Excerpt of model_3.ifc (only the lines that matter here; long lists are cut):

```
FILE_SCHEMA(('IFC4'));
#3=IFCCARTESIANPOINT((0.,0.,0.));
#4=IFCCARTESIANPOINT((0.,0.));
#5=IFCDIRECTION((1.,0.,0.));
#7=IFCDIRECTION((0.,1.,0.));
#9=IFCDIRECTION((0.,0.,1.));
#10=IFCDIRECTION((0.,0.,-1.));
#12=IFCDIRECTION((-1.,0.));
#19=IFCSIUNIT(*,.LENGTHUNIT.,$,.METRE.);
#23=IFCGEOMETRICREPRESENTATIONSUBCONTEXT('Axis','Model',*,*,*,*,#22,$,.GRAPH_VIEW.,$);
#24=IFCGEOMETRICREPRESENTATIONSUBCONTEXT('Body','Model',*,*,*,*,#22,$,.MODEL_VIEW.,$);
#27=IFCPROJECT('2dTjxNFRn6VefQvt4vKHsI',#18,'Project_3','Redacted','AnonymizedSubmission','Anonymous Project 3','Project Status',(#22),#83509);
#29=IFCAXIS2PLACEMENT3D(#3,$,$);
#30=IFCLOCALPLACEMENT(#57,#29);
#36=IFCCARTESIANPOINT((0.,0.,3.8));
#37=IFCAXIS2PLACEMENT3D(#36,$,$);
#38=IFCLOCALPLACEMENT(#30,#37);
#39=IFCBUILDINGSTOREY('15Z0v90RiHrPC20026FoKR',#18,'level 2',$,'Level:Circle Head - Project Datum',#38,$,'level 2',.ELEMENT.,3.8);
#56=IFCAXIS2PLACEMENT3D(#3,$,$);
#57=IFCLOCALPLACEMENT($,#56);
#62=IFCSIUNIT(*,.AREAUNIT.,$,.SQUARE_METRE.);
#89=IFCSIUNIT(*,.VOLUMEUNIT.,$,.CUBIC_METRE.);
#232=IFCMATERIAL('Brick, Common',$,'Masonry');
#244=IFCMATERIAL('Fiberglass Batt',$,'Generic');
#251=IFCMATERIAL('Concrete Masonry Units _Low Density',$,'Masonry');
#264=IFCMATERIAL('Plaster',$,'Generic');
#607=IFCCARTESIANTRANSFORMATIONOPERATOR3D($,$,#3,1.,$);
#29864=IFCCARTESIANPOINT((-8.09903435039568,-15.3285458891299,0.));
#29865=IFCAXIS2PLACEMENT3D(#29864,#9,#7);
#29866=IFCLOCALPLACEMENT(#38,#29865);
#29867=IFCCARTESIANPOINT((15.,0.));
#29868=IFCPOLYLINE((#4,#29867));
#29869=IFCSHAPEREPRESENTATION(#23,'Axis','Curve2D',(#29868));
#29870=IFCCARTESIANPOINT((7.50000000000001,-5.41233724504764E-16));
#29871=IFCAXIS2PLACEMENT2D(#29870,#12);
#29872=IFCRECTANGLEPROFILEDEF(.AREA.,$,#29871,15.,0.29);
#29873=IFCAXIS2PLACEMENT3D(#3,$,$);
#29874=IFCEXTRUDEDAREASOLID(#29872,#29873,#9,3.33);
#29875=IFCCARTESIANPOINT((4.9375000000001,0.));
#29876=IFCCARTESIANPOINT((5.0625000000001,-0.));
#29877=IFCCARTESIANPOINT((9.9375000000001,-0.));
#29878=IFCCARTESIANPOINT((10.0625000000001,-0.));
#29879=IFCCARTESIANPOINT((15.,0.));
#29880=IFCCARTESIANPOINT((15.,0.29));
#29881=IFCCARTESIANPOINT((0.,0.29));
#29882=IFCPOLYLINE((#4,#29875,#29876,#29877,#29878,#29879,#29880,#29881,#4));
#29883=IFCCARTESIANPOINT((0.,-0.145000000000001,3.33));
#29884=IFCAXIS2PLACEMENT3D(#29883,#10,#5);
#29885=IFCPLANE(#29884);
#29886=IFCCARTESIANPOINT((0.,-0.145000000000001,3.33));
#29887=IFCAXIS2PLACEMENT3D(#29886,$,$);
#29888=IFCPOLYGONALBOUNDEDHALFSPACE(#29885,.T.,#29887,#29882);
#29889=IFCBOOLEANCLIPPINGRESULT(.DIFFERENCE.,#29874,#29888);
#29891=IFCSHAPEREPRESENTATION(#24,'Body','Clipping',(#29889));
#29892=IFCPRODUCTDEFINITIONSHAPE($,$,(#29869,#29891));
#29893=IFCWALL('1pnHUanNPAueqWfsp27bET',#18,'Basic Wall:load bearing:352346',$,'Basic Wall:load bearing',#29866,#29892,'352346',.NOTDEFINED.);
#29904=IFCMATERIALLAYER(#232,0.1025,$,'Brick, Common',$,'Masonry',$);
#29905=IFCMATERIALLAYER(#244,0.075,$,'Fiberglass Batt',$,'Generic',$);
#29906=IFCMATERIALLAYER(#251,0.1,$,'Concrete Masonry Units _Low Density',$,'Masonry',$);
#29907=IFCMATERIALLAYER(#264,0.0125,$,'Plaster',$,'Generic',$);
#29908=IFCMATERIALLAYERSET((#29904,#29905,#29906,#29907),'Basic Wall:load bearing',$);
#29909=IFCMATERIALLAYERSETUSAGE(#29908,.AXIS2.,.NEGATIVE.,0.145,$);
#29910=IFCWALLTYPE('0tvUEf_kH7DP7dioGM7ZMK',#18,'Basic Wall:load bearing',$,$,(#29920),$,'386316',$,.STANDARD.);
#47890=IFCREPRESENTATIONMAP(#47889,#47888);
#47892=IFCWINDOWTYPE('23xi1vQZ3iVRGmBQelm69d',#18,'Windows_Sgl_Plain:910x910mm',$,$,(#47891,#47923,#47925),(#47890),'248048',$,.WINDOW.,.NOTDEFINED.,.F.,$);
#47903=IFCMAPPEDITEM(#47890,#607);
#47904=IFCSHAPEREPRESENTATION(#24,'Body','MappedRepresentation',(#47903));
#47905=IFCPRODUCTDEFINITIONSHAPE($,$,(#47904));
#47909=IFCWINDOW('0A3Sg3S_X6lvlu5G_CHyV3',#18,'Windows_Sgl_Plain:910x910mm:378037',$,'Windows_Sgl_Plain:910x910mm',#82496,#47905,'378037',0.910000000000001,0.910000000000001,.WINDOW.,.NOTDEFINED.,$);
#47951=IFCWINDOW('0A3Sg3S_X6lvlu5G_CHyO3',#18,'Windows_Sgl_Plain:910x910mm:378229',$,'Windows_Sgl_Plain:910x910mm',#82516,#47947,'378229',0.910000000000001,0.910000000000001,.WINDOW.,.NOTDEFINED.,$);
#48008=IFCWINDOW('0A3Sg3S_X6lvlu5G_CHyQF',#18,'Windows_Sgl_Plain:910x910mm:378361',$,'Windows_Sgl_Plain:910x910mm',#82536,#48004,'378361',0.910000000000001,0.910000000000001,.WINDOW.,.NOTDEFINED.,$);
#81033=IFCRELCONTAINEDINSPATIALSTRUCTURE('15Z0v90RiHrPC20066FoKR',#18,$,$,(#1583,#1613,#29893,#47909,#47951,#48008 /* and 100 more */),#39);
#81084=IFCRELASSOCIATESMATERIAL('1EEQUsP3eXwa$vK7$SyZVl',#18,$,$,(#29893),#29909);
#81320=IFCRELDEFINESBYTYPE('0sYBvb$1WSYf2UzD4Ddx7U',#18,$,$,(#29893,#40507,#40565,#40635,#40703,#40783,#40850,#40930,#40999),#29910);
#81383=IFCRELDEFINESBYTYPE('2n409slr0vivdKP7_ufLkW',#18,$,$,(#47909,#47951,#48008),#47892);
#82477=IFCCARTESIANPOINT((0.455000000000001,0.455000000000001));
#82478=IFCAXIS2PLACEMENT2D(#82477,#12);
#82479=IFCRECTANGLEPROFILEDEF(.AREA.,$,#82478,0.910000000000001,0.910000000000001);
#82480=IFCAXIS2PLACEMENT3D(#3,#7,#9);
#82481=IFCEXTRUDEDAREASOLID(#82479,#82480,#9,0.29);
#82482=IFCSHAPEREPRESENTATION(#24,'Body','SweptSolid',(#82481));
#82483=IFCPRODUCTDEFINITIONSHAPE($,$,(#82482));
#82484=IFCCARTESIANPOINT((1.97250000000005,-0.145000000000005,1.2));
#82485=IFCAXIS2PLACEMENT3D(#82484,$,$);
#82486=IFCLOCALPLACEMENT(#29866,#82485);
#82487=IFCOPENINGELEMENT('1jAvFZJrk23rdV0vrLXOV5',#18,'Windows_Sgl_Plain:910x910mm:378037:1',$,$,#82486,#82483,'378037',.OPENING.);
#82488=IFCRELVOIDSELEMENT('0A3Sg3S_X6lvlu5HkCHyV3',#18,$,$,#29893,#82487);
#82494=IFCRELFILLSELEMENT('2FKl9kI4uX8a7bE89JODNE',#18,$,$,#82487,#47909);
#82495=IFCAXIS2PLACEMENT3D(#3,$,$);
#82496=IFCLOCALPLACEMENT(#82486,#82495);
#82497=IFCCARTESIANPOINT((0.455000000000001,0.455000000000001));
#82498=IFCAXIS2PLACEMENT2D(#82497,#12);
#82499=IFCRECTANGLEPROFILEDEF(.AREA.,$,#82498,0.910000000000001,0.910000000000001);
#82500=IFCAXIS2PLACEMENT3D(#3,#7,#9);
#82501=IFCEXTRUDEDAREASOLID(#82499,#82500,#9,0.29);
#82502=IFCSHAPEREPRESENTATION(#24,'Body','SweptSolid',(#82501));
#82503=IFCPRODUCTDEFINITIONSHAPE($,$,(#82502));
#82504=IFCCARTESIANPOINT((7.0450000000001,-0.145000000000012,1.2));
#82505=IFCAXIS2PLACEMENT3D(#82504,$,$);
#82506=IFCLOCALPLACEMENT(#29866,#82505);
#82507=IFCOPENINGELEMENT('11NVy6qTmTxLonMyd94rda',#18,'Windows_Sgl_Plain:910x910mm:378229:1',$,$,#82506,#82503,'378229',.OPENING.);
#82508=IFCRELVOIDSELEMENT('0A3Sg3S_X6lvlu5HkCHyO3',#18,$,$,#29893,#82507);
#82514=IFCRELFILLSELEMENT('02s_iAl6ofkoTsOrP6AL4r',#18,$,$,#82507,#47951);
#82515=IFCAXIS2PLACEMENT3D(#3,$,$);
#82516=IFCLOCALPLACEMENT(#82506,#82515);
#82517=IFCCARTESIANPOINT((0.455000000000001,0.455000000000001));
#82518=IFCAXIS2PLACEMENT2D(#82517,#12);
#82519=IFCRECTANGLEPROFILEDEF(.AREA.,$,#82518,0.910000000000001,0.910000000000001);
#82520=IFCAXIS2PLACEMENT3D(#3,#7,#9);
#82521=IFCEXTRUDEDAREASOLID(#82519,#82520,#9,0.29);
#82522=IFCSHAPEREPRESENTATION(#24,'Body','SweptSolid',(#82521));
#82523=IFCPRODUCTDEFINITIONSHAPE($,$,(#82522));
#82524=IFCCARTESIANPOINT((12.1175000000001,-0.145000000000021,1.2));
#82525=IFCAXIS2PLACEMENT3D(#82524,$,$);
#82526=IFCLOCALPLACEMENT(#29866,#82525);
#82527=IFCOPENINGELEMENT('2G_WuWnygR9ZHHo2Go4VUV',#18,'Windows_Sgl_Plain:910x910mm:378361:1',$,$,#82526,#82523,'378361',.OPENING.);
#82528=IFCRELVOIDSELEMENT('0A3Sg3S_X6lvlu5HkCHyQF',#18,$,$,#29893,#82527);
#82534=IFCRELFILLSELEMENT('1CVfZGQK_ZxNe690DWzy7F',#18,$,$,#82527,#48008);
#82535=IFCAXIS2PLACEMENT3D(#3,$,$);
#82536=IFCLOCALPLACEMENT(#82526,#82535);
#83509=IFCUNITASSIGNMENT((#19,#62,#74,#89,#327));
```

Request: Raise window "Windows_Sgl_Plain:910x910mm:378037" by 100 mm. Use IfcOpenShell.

```python
import numpy as np
import ifcopenshell
import ifcopenshell.api.geometry
import ifcopenshell.util.placement
import ifcopenshell.util.unit

model = ifcopenshell.open("model_3.ifc")
unit_scale = ifcopenshell.util.unit.calculate_unit_scale(model)

window = model.by_guid("0A3Sg3S_X6lvlu5G_CHyV3")
opening = window.FillsVoids[0].RelatingOpeningElement
dz = 0.1 / unit_scale

shift = np.array([0.0, 0.0, dz])
# The window is placed relative to its opening, so it follows when the opening moves.
matrix = ifcopenshell.util.placement.get_local_placement(opening.ObjectPlacement)
matrix[:3, 3] += shift
ifcopenshell.api.geometry.edit_object_placement(
    model, product=opening, matrix=matrix, is_si=False, should_transform_children=True
)

print(f"moved by {dz * unit_scale:+.3f} m")

model.write("model_3-out.ifc")
```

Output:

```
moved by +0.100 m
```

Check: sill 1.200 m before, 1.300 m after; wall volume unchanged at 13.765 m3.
